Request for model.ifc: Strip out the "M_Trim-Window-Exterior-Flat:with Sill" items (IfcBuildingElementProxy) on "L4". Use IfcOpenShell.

First a look at what the model holds.

```python
import ifcopenshell
import ifcopenshell.util.element

model = ifcopenshell.open("model.ifc")
print(model.schema)
storey = next(s for s in model.by_type("IfcBuildingStorey") if s.Name == "L4")
proxies = [e for e in ifcopenshell.util.element.get_decomposition(storey) if e.is_a("IfcBuildingElementProxy")]
seen = {}
for e in proxies:
    element_type = ifcopenshell.util.element.get_type(e)
    name = element_type.Name if element_type not in (None, e) else None
    seen[name] = seen.get(name, 0) + 1
for name, count in sorted(seen.items(), key=str):
    print(count, "x", name)
```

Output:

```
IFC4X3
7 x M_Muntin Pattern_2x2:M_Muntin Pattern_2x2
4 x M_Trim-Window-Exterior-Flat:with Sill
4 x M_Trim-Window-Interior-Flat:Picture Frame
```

```python
import ifcopenshell
import ifcopenshell.api.root
import ifcopenshell.util.element

model = ifcopenshell.open("model.ifc")

storey = next(s for s in model.by_type("IfcBuildingStorey") if s.Name == "L4")
proxies = [e for e in ifcopenshell.util.element.get_decomposition(storey) if e.is_a("IfcBuildingElementProxy")]
targets = [e for e in proxies if (t := ifcopenshell.util.element.get_type(e)) not in (None, e) and t.Name == "M_Trim-Window-Exterior-Flat:with Sill"]

for e in targets:
    ifcopenshell.api.root.remove_product(model, product=e)
print(len(targets), "removed")

model.write("model_rev.ifc")
```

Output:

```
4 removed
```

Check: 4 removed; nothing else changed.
